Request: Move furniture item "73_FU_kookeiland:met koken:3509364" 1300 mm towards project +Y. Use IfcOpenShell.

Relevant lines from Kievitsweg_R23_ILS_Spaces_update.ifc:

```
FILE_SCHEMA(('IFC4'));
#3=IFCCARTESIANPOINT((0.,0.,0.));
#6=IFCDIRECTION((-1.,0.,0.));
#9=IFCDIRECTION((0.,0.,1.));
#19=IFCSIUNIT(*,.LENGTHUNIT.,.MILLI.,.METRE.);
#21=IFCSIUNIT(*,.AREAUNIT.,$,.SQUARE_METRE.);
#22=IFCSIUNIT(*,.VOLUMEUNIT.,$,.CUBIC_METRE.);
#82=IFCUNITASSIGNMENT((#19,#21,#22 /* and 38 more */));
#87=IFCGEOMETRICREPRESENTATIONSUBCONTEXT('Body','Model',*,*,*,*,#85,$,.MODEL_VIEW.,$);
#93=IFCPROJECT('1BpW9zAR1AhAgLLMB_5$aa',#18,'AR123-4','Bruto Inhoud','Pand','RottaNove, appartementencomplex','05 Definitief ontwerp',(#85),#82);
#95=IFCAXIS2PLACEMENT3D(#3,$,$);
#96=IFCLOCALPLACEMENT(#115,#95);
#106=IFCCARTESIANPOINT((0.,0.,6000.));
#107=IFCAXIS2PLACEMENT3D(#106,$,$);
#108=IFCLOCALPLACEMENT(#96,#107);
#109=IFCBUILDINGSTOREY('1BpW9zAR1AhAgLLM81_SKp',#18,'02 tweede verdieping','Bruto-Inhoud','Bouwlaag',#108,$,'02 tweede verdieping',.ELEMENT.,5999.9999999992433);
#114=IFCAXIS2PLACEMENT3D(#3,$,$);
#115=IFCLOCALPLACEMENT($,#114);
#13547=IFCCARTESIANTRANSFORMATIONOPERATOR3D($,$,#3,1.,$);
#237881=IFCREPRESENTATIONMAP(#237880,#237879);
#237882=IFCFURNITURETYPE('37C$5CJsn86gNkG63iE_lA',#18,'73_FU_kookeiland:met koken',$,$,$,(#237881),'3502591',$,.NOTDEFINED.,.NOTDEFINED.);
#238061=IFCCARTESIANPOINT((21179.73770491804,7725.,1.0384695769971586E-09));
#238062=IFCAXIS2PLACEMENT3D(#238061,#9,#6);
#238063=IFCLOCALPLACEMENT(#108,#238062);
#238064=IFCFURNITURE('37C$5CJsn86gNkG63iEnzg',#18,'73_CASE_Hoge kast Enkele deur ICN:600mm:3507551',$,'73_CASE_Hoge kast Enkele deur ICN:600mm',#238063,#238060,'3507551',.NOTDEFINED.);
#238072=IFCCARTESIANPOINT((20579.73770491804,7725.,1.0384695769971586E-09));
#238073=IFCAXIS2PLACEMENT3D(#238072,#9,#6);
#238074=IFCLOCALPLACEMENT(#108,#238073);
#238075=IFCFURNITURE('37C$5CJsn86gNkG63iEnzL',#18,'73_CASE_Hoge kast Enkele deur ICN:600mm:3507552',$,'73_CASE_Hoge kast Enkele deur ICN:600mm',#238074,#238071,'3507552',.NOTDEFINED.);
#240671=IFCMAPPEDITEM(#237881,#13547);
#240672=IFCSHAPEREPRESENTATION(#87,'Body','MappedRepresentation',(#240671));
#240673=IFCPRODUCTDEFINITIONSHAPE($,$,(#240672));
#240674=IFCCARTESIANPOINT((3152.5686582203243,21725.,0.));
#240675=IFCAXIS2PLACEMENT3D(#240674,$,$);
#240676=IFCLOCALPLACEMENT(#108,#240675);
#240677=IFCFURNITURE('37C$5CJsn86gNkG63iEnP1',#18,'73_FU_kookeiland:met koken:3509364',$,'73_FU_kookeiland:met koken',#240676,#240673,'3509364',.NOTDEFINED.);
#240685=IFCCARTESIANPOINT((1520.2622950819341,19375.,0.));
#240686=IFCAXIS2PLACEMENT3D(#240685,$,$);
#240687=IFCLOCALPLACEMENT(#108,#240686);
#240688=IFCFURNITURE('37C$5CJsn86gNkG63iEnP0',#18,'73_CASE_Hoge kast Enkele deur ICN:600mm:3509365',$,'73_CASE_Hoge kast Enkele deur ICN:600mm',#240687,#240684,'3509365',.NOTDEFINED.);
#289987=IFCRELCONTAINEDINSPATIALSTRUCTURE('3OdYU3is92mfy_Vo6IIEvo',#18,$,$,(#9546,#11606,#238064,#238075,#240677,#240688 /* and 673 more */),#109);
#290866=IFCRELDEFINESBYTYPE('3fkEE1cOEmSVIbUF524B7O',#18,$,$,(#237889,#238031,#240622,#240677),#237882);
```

```python
import ifcopenshell
import ifcopenshell.api.geometry
import ifcopenshell.util.placement
import ifcopenshell.util.unit

model = ifcopenshell.open("Kievitsweg_R23_ILS_Spaces_update.ifc")
unit_scale = ifcopenshell.util.unit.calculate_unit_scale(model)

item = model.by_guid("37C$5CJsn86gNkG63iEnP1")
matrix = ifcopenshell.util.placement.get_local_placement(item.ObjectPlacement)
matrix[1, 3] += 1.3 / unit_scale
ifcopenshell.api.geometry.edit_object_placement(model, product=item, matrix=matrix, is_si=False)

print(ifcopenshell.util.placement.get_local_placement(item.ObjectPlacement).round(3) + 0.0)

model.write("Kievitsweg_R23_ILS_Spaces_update_rev.ifc")
```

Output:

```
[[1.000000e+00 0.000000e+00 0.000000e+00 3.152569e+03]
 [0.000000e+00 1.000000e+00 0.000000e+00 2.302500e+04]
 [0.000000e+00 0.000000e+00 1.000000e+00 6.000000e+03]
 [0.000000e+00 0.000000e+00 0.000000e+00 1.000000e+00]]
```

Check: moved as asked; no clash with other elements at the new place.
